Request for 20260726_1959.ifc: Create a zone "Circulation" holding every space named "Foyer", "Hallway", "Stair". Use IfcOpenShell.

First a look at what the model holds.

```python
import ifcopenshell

model = ifcopenshell.open("20260726_1959.ifc")
print(model.schema)
seen = {}
for space in model.by_type("IfcSpace"):
    seen[space.LongName] = seen.get(space.LongName, 0) + 1
for name, count in sorted(seen.items(), key=str):
    print(count, "x", name)
print("zones:", [z.Name for z in model.by_type("IfcZone")][:20])
```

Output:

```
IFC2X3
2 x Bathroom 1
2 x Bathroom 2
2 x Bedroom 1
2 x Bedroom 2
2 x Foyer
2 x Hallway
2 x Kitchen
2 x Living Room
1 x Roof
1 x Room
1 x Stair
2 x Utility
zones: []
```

```python
import ifcopenshell
import ifcopenshell.api.group
import ifcopenshell.api.root

model = ifcopenshell.open("20260726_1959.ifc")

names = {"Foyer", "Hallway", "Stair"}
spaces = [s for s in model.by_type("IfcSpace") if s.LongName in names]

zone = ifcopenshell.api.root.create_entity(model, ifc_class="IfcZone", name="Circulation")
ifcopenshell.api.group.assign_group(model, products=spaces, group=zone)
print(len(spaces), "spaces in", zone.Name)

model.write("20260726_1959_edited.ifc")
```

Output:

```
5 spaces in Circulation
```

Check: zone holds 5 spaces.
